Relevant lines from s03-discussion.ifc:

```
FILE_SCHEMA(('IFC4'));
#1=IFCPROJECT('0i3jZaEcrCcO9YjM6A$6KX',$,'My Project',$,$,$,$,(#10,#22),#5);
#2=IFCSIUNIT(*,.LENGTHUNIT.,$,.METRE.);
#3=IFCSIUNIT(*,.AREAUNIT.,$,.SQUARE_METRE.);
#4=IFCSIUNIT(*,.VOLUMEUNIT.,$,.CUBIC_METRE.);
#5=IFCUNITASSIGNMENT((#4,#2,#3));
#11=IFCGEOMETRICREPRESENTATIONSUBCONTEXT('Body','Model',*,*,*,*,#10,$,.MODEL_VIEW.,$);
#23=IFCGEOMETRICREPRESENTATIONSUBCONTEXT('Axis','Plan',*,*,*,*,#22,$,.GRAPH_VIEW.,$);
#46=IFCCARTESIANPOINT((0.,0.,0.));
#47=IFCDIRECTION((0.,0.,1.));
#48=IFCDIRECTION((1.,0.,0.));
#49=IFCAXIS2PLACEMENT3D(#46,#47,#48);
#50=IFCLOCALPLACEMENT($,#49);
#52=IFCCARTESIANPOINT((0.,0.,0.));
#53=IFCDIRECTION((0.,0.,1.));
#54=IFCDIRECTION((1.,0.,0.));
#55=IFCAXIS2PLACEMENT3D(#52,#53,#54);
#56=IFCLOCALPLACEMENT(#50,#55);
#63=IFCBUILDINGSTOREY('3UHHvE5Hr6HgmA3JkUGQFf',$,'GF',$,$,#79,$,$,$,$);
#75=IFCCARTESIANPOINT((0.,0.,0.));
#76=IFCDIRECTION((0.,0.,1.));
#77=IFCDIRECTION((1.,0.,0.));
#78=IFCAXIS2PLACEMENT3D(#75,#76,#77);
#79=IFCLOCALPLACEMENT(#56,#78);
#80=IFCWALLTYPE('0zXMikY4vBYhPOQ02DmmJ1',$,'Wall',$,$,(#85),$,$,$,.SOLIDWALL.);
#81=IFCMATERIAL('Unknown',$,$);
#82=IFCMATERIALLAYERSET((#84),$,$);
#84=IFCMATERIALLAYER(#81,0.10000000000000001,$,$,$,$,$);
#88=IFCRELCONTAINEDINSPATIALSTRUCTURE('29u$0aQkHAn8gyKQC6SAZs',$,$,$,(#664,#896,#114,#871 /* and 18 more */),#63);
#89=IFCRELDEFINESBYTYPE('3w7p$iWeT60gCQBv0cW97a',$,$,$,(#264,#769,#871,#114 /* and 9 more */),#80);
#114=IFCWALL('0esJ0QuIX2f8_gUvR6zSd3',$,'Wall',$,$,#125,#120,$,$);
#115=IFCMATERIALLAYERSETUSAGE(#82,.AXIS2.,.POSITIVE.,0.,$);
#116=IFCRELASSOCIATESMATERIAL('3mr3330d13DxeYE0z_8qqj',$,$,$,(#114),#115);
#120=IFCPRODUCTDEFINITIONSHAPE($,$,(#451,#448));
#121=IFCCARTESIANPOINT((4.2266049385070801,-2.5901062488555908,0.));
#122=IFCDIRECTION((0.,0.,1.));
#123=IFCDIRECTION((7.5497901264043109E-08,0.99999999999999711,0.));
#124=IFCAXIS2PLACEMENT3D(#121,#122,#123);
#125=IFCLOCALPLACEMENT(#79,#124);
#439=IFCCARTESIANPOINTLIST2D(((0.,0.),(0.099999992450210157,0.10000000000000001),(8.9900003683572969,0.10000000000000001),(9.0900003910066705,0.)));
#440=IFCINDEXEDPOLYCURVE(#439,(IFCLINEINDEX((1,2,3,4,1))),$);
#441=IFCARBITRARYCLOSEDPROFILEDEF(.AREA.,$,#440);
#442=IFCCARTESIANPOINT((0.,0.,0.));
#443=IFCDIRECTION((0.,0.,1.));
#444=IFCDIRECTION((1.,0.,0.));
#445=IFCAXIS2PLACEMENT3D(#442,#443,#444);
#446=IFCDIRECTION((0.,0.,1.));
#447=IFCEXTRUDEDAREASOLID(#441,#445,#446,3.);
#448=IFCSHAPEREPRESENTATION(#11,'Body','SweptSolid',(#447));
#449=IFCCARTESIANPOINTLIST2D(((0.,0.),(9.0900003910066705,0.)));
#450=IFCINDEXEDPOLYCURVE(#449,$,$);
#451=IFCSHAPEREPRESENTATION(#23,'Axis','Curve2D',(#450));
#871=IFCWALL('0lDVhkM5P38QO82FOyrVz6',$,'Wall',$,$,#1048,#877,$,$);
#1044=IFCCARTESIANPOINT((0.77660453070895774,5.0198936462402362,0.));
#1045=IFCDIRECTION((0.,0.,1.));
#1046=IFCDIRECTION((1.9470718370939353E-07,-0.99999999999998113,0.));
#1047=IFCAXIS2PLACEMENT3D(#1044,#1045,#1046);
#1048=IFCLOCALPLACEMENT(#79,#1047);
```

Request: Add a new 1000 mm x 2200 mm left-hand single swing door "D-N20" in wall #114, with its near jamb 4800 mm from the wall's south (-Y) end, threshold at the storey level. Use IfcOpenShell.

```python
import numpy as np
import ifcopenshell
import ifcopenshell.api.feature
import ifcopenshell.api.geometry
import ifcopenshell.api.root
import ifcopenshell.api.spatial
import ifcopenshell.geom
import ifcopenshell.util.element
import ifcopenshell.util.placement
import ifcopenshell.util.representation
import ifcopenshell.util.shape
import ifcopenshell.util.unit

model = ifcopenshell.open("s03-discussion.ifc")
unit_scale = ifcopenshell.util.unit.calculate_unit_scale(model)
settings = ifcopenshell.geom.settings()


def volume(element):
    """Net volume in cubic metres, openings subtracted."""
    shape = ifcopenshell.geom.create_shape(settings, element)
    return ifcopenshell.util.shape.get_volume(shape.geometry)


wall = model.by_id(114)
storey = ifcopenshell.util.element.get_container(wall, ifc_class="IfcBuildingStorey")
context = ifcopenshell.util.representation.get_context(model, "Model", "Body", "MODEL_VIEW")
before = volume(wall)

width, height, from_end, sill = 1, 2.2, 4.8, 0.0  # metres

# The wall runs along its own X axis, and the end named is its -X end.
wall_shape = ifcopenshell.geom.create_shape(settings, wall)
x, y, z = ifcopenshell.util.shape.get_vertices(wall_shape.geometry).T
start = x.min() + from_end
face, thickness = float(y.min()), float(y.max() - y.min())
wall_matrix = ifcopenshell.util.placement.get_local_placement(wall.ObjectPlacement)
level = ifcopenshell.util.placement.get_local_placement(storey.ObjectPlacement)[2, 3]


def in_wall(x, y):
    """Placement at x, y metres in the wall's axes, at sill height."""
    matrix = wall_matrix.copy()
    matrix[:, 3] = wall_matrix @ np.array([x / unit_scale, y / unit_scale, 0.0, 1.0])
    matrix[2, 3] = level + sill / unit_scale
    return matrix


# Opening: a box that overshoots both wall faces by 50 mm.
opening = ifcopenshell.api.root.create_entity(model, ifc_class="IfcOpeningElement", predefined_type="OPENING")
box = ifcopenshell.api.geometry.add_wall_representation(
    model, context=context, length=width, height=height, thickness=thickness + 0.1
)
ifcopenshell.api.geometry.assign_representation(model, product=opening, representation=box)
ifcopenshell.api.geometry.edit_object_placement(model, product=opening, matrix=in_wall(start, face - 0.05), is_si=False)
ifcopenshell.api.feature.add_feature(model, feature=opening, element=wall)

door = ifcopenshell.api.root.create_entity(model, ifc_class="IfcDoor", name="D-N20", predefined_type="DOOR")
door.OverallWidth, door.OverallHeight = width / unit_scale, height / unit_scale
door.OperationType = "SINGLE_SWING_LEFT"
body = ifcopenshell.api.geometry.add_door_representation(
    model,
    context=context,
    overall_width=door.OverallWidth,
    overall_height=door.OverallHeight,
    operation_type="SINGLE_SWING_LEFT",
    lining_properties={"LiningDepth": thickness / unit_scale, "ThresholdDepth": thickness / unit_scale},
)
ifcopenshell.api.geometry.assign_representation(model, product=door, representation=body)
ifcopenshell.api.spatial.assign_container(model, products=[door], relating_structure=storey)
ifcopenshell.api.feature.add_filling(model, opening=opening, element=door)

# The lining spans the wall, so the door starts at the wall face.
ifcopenshell.api.geometry.edit_object_placement(model, product=door, matrix=in_wall(start, face), is_si=False)

after = volume(wall)

print(f"wall volume {before:.3f} -> {after:.3f} m3")

model.write("s03-discussion_edited.ifc")
```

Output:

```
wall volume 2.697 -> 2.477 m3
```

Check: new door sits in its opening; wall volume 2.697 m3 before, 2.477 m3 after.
